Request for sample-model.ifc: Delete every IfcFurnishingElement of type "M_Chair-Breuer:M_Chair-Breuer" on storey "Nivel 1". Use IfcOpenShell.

First a look at what the model holds.

```python
import ifcopenshell
import ifcopenshell.util.element

model = ifcopenshell.open("sample-model.ifc")
print(model.schema)
storey = next(s for s in model.by_type("IfcBuildingStorey") if s.Name == "Nivel 1")
furniture = [e for e in ifcopenshell.util.element.get_decomposition(storey) if e.is_a("IfcFurnishingElement")]
seen = {}
for e in furniture:
    element_type = ifcopenshell.util.element.get_type(e)
    name = element_type.Name if element_type not in (None, e) else None
    seen[name] = seen.get(name, 0) + 1
for name, count in sorted(seen.items(), key=str):
    print(count, "x", name)
```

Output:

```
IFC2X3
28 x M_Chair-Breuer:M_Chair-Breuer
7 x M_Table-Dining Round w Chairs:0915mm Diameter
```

```python
import ifcopenshell
import ifcopenshell.api.root
import ifcopenshell.util.element

model = ifcopenshell.open("sample-model.ifc")

storey = next(s for s in model.by_type("IfcBuildingStorey") if s.Name == "Nivel 1")
furniture = [e for e in ifcopenshell.util.element.get_decomposition(storey) if e.is_a("IfcFurnishingElement")]
targets = [e for e in furniture if (t := ifcopenshell.util.element.get_type(e)) not in (None, e) and t.Name == "M_Chair-Breuer:M_Chair-Breuer"]

for e in targets:
    ifcopenshell.api.root.remove_product(model, product=e)
print(len(targets), "removed")

model.write("sample-model_updated.ifc")
```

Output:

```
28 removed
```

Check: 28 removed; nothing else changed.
